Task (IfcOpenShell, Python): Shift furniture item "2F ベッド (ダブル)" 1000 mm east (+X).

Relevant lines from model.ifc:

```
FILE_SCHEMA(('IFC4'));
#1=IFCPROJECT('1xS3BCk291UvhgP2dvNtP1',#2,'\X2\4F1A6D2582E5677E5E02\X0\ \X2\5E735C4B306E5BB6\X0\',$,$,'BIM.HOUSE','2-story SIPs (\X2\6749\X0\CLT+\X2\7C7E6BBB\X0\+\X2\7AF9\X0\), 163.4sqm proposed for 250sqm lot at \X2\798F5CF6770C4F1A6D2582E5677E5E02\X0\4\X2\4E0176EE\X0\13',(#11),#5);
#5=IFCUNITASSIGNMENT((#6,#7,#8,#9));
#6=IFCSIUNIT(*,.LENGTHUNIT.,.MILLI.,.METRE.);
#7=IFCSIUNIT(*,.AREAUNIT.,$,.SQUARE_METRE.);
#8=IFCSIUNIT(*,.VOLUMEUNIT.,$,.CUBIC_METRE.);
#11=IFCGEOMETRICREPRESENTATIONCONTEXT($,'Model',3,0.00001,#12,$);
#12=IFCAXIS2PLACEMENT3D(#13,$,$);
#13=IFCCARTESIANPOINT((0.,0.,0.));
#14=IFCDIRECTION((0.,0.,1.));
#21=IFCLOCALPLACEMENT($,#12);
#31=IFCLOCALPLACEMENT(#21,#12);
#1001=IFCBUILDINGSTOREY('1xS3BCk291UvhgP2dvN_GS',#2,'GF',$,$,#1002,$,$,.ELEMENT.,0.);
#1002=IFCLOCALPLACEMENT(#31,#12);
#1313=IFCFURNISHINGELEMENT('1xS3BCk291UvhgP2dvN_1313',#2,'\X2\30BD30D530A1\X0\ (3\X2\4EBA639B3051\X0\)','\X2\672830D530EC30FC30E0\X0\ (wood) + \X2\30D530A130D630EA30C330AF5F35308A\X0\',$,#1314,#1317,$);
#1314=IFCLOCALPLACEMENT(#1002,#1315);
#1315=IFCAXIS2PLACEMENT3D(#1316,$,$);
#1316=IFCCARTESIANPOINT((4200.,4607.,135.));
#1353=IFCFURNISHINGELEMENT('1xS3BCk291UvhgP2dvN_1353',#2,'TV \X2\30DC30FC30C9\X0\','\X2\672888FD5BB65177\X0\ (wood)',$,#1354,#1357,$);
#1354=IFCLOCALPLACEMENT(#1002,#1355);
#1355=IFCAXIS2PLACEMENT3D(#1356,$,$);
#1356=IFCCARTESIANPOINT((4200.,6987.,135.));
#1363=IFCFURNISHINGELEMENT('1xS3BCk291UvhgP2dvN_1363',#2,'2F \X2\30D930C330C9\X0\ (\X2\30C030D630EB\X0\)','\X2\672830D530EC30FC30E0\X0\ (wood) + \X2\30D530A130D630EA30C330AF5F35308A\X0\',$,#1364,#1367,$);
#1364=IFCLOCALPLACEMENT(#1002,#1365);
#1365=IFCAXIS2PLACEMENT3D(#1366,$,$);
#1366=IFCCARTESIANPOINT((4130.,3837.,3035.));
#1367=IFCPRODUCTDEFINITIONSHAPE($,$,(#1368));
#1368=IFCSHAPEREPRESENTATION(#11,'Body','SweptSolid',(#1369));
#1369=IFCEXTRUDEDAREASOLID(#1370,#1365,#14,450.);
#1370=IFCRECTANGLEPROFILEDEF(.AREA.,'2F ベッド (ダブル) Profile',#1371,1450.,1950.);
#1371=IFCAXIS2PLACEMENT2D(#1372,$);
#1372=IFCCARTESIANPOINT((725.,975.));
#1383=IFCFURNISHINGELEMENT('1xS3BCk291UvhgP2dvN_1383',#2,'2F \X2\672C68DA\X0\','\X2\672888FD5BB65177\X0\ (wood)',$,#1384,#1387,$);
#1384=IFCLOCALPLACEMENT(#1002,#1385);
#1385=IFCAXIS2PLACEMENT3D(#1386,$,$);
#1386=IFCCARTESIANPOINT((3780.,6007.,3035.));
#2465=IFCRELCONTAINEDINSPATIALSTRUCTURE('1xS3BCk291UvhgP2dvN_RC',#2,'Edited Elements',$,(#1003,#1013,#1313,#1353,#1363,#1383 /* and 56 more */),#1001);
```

```python
import ifcopenshell
import ifcopenshell.api.geometry
import ifcopenshell.util.placement

model = ifcopenshell.open("model.ifc")

item = model.by_guid("1xS3BCk291UvhgP2dvN_1363")
matrix = ifcopenshell.util.placement.get_local_placement(item.ObjectPlacement)
matrix[0, 3] += 1000.0
ifcopenshell.api.geometry.edit_object_placement(model, product=item, matrix=matrix, is_si=False)

print(ifcopenshell.util.placement.get_local_placement(item.ObjectPlacement).round(3) + 0.0)

model.write("model-out.ifc")
```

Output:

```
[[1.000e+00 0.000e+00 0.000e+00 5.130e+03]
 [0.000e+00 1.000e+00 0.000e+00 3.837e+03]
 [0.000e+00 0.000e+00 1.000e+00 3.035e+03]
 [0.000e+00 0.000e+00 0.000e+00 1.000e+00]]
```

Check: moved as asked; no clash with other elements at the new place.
